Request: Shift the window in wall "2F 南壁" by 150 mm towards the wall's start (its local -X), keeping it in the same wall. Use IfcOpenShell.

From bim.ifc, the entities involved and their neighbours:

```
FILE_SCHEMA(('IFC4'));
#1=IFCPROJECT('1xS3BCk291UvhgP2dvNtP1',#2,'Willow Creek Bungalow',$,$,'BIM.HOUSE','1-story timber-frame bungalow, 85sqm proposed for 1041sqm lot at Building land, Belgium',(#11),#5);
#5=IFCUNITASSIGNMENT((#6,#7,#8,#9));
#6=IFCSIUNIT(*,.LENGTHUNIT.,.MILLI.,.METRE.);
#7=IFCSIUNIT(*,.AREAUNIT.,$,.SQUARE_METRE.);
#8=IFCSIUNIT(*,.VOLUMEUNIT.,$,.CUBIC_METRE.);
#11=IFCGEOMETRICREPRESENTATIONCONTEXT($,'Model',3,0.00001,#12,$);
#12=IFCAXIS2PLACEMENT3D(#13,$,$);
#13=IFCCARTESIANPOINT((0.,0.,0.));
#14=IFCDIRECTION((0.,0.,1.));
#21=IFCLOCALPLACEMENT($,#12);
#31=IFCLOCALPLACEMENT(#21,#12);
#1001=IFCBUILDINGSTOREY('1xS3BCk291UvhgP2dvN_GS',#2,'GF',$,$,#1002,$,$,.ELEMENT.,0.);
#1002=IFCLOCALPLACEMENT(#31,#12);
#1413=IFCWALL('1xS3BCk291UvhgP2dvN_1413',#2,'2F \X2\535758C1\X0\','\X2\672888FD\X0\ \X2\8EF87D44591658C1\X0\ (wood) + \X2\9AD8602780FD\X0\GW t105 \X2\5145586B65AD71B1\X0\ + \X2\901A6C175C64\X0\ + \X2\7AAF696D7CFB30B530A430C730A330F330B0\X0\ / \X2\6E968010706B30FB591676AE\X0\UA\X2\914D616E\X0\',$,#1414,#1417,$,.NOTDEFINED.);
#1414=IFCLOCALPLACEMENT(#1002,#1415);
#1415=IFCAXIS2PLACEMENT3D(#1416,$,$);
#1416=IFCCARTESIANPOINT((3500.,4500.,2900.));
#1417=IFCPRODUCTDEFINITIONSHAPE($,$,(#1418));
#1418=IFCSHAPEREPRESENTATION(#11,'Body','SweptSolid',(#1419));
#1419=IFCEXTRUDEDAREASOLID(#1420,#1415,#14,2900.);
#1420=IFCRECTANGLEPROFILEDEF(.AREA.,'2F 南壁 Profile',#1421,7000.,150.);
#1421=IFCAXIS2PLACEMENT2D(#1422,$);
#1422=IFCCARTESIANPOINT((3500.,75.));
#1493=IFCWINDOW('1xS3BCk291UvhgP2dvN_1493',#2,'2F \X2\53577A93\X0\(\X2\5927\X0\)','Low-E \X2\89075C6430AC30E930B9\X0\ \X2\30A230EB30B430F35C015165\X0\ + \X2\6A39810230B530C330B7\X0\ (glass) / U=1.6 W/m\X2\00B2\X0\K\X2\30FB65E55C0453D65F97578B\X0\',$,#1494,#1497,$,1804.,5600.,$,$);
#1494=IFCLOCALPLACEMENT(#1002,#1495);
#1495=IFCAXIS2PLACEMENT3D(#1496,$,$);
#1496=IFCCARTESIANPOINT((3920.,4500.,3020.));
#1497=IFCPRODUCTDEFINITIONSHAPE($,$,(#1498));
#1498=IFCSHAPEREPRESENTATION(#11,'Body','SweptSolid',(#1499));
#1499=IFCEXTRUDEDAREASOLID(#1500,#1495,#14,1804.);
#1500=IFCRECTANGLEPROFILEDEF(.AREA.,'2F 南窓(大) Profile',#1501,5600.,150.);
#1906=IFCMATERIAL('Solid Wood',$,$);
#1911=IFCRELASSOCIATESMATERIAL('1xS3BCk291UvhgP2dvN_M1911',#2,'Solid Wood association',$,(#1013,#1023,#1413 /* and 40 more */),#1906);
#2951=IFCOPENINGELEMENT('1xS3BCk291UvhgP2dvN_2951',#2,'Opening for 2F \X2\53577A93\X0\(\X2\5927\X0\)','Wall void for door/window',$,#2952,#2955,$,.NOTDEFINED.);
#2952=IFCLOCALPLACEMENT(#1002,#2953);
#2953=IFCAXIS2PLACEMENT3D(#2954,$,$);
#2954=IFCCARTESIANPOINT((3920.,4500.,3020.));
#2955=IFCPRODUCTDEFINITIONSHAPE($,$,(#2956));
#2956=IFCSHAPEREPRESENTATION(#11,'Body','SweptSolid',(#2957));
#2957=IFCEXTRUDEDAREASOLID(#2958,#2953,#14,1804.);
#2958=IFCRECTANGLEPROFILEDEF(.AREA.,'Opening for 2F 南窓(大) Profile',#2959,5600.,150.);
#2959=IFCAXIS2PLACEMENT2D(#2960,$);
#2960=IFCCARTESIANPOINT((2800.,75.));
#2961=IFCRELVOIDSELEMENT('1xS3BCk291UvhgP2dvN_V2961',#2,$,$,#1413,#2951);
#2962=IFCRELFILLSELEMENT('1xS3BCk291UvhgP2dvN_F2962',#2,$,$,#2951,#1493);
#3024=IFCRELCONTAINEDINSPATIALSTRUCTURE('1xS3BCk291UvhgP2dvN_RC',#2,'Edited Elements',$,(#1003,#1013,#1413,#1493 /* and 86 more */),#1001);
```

```python
import ifcopenshell
import ifcopenshell.api.geometry
import ifcopenshell.util.placement

model = ifcopenshell.open("bim.ifc")

window = model.by_guid("1xS3BCk291UvhgP2dvN_1493")
opening = window.FillsVoids[0].RelatingOpeningElement
wall = opening.VoidsElements[0].RelatingBuildingElement

wall_matrix = ifcopenshell.util.placement.get_local_placement(wall.ObjectPlacement)
shift = wall_matrix[:3, 0] * -150.0
before = ifcopenshell.util.placement.get_local_placement(window.ObjectPlacement)[:3, 3].copy()

# The window is not placed relative to its opening, so move both.
for product in (opening, window):
    matrix = ifcopenshell.util.placement.get_local_placement(product.ObjectPlacement)
    matrix[:3, 3] += shift
    ifcopenshell.api.geometry.edit_object_placement(model, product=product, matrix=matrix, is_si=False)

after = ifcopenshell.util.placement.get_local_placement(window.ObjectPlacement)[:3, 3]
print("window moved by", (after - before).round(3) + 0.0)

model.write("bim_edited.ifc")
```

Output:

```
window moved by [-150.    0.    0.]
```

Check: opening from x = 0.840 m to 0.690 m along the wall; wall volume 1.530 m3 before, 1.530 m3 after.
